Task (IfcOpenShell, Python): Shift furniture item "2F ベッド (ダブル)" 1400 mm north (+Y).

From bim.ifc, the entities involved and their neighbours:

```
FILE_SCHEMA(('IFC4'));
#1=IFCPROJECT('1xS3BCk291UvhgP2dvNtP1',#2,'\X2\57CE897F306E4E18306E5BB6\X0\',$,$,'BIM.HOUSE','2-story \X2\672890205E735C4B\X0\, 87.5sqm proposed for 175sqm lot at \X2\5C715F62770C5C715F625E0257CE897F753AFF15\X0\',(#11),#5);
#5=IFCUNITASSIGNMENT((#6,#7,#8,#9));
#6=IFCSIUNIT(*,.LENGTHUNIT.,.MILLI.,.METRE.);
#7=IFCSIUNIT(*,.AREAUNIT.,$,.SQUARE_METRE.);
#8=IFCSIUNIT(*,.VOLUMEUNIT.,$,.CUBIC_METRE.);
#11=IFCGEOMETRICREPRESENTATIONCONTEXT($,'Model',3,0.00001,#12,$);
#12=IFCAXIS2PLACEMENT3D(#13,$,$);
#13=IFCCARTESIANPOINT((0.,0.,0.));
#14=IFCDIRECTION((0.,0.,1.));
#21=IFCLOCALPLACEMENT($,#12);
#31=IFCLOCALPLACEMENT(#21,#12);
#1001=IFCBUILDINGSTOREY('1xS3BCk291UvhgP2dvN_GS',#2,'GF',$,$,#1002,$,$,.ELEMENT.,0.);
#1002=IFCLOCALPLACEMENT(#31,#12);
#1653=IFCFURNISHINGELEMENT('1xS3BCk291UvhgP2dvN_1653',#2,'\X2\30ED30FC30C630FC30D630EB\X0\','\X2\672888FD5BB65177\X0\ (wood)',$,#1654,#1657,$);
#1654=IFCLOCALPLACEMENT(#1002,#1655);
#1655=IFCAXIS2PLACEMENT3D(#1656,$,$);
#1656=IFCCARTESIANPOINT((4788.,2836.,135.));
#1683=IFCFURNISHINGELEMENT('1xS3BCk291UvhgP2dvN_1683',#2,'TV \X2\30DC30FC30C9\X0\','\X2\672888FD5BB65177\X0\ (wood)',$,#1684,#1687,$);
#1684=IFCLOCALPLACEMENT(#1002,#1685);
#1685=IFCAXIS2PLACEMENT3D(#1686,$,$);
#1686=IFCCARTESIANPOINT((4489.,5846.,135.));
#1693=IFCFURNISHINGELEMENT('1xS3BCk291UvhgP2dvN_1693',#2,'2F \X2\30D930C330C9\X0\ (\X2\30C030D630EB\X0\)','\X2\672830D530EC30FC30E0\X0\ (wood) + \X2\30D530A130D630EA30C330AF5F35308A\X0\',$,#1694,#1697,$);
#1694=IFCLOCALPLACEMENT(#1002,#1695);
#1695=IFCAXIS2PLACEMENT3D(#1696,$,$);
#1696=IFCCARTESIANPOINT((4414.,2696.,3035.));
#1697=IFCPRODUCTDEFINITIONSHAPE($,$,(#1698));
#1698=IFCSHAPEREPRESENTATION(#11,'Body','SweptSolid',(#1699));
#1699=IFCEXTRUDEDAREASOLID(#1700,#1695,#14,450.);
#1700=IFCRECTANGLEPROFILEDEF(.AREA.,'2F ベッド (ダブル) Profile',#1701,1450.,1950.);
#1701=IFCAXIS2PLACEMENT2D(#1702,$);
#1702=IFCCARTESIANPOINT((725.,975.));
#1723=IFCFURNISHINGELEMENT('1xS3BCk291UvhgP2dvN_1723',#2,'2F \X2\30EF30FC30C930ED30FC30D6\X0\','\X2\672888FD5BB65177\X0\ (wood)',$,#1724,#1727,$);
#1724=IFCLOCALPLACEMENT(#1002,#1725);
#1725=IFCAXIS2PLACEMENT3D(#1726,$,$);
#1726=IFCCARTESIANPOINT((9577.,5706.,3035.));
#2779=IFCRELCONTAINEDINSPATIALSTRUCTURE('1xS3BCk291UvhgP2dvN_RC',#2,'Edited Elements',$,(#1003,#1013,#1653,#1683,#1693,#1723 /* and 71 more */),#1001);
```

```python
import ifcopenshell
import ifcopenshell.api.geometry
import ifcopenshell.util.placement

model = ifcopenshell.open("bim.ifc")

item = model.by_id(1693)
matrix = ifcopenshell.util.placement.get_local_placement(item.ObjectPlacement)
matrix[1, 3] += 1400.0
ifcopenshell.api.geometry.edit_object_placement(model, product=item, matrix=matrix, is_si=False)

print(ifcopenshell.util.placement.get_local_placement(item.ObjectPlacement).round(3) + 0.0)

model.write("bim_edited.ifc")
```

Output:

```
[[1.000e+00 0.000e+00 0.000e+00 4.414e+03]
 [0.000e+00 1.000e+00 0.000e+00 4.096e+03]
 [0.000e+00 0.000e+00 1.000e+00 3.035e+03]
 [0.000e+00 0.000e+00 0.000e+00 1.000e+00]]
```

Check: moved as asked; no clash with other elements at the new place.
